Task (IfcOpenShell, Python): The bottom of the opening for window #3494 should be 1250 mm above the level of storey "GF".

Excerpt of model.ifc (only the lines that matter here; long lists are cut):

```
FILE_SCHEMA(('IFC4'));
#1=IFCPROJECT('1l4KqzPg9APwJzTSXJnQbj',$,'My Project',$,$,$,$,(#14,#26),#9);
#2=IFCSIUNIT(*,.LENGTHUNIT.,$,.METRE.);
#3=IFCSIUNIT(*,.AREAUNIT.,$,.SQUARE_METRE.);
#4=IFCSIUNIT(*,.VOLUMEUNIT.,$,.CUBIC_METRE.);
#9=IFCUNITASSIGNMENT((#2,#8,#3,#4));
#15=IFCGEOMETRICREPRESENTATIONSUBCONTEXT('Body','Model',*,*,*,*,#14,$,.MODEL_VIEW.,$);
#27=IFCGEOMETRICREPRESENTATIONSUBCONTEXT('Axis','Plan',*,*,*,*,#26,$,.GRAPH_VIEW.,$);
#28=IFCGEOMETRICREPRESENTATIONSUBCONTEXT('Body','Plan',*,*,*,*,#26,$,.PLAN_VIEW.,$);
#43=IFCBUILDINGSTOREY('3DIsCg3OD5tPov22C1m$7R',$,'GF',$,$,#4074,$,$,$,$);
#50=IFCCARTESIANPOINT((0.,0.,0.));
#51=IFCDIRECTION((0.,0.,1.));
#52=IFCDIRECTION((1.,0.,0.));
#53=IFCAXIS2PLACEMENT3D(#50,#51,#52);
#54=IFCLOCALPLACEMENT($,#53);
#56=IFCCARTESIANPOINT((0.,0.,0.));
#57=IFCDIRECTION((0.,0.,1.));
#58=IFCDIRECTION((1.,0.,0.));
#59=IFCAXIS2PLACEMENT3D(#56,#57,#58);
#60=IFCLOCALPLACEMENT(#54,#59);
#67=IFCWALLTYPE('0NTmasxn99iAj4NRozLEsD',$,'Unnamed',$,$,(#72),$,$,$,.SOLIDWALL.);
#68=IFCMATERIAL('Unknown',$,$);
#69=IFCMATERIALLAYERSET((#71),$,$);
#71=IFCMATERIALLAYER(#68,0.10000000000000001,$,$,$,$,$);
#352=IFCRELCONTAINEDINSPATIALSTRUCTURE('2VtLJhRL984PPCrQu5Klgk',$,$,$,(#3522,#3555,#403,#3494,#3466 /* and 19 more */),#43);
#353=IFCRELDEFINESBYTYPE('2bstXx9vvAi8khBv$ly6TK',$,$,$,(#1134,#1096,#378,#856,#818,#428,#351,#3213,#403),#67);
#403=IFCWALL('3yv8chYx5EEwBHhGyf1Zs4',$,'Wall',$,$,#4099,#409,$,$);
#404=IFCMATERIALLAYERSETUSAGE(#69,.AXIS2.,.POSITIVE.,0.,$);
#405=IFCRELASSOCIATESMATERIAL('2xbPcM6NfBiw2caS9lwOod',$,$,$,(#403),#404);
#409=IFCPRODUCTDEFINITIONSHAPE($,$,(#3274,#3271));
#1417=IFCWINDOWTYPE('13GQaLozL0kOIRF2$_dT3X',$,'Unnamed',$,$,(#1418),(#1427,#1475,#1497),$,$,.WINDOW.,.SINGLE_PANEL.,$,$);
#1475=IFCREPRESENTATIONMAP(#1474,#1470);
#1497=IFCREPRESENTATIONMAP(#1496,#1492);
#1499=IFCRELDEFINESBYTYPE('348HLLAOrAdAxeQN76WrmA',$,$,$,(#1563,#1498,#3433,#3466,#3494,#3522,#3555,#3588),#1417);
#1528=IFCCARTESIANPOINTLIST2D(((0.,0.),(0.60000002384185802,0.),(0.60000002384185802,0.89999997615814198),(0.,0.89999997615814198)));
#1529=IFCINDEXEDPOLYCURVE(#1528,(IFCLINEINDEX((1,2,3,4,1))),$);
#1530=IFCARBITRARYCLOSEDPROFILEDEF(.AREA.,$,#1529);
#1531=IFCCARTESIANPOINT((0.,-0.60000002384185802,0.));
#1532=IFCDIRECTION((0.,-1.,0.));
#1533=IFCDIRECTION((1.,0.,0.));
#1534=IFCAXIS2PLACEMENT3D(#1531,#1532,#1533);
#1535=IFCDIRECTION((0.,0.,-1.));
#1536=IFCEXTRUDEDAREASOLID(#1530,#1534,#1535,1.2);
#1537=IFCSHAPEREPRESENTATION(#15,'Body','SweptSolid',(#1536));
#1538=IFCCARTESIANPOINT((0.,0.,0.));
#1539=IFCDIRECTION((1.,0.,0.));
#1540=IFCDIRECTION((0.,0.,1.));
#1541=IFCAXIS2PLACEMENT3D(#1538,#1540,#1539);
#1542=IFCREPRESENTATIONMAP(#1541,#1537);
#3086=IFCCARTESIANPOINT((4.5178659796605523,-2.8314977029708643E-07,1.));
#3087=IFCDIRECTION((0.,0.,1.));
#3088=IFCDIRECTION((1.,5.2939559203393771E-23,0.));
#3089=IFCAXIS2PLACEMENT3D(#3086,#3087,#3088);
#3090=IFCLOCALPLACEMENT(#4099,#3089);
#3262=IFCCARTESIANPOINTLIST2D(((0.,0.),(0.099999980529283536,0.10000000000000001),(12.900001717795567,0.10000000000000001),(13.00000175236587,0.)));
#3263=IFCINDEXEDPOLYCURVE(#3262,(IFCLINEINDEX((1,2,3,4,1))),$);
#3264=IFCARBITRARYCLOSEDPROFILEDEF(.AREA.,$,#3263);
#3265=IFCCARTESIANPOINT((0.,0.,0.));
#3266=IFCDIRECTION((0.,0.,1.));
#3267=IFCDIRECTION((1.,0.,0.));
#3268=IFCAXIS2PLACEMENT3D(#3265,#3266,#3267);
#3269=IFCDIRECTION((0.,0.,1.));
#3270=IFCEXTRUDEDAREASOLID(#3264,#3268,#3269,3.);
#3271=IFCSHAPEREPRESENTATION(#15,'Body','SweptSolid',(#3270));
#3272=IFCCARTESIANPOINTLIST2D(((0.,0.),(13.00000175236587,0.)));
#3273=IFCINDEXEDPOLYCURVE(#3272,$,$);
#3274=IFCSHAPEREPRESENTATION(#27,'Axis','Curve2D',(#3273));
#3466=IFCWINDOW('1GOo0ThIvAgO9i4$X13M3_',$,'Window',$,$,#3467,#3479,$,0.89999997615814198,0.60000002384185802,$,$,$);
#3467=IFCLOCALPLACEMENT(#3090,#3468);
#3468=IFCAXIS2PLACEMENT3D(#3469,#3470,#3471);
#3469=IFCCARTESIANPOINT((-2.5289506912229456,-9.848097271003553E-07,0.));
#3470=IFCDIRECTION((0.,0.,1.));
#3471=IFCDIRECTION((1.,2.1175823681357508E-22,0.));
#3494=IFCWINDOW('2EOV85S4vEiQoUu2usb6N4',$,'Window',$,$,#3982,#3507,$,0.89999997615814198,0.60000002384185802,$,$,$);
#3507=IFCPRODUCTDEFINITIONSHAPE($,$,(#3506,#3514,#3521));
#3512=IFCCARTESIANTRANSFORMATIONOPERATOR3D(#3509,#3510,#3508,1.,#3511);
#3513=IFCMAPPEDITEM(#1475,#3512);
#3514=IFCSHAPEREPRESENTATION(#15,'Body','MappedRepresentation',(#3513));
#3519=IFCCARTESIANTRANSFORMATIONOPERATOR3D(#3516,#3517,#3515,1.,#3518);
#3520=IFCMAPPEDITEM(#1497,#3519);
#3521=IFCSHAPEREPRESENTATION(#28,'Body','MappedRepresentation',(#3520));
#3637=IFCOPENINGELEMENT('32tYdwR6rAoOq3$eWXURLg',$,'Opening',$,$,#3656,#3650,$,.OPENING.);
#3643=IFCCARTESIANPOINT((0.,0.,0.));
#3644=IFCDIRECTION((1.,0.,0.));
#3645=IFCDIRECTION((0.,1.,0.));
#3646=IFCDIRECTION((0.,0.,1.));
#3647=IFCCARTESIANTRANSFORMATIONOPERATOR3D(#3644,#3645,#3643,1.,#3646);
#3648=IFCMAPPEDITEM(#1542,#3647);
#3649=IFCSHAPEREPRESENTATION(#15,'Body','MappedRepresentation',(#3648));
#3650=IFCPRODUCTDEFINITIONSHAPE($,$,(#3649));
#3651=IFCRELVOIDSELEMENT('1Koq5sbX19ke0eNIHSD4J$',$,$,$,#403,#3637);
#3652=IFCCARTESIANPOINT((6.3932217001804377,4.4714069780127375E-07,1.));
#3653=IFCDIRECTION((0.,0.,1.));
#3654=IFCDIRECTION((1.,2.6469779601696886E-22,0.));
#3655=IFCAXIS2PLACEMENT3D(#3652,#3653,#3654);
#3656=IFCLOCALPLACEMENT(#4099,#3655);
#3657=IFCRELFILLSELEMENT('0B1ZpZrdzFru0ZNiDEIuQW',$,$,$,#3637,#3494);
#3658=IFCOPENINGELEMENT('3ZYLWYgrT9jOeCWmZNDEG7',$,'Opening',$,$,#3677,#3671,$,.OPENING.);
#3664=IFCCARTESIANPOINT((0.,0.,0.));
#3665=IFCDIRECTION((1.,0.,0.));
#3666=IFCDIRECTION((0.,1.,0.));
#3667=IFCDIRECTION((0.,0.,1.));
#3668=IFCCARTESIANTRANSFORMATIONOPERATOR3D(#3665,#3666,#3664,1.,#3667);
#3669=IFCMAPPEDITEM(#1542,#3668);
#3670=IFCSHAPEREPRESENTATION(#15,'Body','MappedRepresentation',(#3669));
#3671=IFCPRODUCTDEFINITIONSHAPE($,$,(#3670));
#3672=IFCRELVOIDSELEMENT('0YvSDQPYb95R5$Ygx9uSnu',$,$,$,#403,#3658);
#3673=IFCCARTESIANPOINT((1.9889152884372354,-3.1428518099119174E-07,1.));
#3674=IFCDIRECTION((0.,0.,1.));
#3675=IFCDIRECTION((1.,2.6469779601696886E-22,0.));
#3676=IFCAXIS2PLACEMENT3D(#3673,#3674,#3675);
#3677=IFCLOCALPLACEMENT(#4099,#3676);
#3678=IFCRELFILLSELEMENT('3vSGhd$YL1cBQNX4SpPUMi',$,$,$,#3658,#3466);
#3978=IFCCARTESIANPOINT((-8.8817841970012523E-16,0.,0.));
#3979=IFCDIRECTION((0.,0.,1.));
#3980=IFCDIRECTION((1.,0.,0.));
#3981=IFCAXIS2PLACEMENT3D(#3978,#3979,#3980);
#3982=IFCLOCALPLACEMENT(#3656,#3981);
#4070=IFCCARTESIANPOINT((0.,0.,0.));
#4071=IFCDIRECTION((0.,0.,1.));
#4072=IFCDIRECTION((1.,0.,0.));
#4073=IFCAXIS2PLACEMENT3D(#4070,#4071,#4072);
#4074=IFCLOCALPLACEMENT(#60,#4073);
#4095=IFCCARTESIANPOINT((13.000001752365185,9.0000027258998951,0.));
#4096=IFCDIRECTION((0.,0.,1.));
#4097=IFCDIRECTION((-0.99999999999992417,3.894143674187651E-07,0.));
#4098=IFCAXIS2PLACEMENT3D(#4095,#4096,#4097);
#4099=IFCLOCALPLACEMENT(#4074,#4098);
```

```python
import numpy as np
import ifcopenshell
import ifcopenshell.api.geometry
import ifcopenshell.geom
import ifcopenshell.util.element
import ifcopenshell.util.placement
import ifcopenshell.util.shape
import ifcopenshell.util.unit

model = ifcopenshell.open("model.ifc")
unit_scale = ifcopenshell.util.unit.calculate_unit_scale(model)

window = model.by_id(3494)
opening = window.FillsVoids[0].RelatingOpeningElement
storey = ifcopenshell.util.element.get_container(window, ifc_class="IfcBuildingStorey")
level = ifcopenshell.util.placement.get_local_placement(storey.ObjectPlacement)[2, 3]

# The opening's origin need not be at the sill, so measure its lowest point.
shape = ifcopenshell.geom.create_shape(ifcopenshell.geom.settings(), opening)
bottom = ifcopenshell.util.shape.get_shape_bottom_elevation(shape, shape.geometry) / unit_scale
dz = level + 1.25 / unit_scale - bottom

shift = np.array([0.0, 0.0, dz])
# The window is placed relative to its opening, so it follows when the opening moves.
matrix = ifcopenshell.util.placement.get_local_placement(opening.ObjectPlacement)
matrix[:3, 3] += shift
ifcopenshell.api.geometry.edit_object_placement(
    model, product=opening, matrix=matrix, is_si=False, should_transform_children=True
)

print(f"moved by {dz * unit_scale:+.3f} m")

model.write("model_edited.ifc")
```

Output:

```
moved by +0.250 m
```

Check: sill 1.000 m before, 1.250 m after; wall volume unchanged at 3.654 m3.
